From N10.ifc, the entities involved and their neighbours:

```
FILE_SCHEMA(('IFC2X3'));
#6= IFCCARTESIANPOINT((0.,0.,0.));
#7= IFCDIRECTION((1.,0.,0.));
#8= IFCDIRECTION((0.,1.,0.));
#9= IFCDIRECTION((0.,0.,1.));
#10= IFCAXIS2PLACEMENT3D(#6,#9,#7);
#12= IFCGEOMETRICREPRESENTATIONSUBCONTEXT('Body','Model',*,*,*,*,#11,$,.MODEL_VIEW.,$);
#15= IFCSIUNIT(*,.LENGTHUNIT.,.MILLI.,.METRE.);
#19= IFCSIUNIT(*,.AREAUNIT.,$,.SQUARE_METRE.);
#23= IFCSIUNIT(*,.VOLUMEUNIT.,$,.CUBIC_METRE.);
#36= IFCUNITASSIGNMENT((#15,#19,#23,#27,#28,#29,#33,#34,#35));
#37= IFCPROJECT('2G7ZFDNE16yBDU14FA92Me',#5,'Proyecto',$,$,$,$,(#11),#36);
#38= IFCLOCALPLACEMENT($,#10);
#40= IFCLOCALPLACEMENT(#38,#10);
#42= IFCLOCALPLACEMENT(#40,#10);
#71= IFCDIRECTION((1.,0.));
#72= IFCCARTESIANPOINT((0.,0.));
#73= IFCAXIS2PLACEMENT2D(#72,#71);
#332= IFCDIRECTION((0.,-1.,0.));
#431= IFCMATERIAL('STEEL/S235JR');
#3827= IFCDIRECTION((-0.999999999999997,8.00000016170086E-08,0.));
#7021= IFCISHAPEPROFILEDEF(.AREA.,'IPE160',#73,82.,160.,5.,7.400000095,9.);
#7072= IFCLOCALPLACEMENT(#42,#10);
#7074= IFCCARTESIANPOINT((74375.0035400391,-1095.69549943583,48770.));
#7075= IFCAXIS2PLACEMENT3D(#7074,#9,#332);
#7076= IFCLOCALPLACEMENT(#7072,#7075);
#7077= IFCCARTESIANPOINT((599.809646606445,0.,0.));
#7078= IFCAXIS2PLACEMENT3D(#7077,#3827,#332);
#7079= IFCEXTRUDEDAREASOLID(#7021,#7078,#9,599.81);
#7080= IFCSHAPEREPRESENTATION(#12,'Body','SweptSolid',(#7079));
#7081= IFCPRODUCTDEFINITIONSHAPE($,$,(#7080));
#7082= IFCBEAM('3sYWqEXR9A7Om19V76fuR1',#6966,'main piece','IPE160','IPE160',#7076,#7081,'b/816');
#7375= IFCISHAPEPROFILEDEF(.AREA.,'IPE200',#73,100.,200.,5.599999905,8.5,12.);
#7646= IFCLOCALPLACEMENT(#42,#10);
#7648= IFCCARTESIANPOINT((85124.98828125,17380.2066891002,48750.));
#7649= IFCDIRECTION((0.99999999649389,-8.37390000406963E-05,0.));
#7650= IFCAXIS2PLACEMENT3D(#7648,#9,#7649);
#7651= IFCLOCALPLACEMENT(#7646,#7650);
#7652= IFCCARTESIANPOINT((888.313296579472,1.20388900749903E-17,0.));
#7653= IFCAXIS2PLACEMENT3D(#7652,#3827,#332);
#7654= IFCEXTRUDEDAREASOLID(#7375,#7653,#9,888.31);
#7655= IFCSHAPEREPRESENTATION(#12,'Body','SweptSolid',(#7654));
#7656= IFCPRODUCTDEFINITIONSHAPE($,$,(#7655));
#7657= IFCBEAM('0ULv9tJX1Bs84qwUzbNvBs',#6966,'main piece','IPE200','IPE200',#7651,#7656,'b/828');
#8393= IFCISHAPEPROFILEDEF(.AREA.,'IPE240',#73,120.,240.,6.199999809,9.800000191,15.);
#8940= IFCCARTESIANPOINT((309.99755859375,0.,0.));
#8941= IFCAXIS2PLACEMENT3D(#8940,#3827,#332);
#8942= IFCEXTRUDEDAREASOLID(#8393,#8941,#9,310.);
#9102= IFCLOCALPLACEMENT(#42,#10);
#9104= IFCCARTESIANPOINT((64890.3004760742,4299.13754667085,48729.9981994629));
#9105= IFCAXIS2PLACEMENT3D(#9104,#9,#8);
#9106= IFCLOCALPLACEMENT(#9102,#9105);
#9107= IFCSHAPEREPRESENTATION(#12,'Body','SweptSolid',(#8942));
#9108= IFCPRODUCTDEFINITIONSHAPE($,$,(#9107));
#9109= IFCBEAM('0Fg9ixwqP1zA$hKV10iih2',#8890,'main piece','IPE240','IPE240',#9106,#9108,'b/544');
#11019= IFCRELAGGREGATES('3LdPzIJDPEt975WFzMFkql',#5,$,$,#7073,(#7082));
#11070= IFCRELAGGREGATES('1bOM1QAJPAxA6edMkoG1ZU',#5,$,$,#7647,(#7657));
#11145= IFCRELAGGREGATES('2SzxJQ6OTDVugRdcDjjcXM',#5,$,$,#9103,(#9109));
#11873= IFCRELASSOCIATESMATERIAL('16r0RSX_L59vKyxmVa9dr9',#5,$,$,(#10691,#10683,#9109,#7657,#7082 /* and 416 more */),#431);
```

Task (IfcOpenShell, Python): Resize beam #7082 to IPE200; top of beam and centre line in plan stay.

```python
import ifcopenshell
import ifcopenshell.util.element
import ifcopenshell.util.representation

model = ifcopenshell.open("N10.ifc")

member = model.by_guid("3sYWqEXR9A7Om19V76fuR1")
source = next(p for p in model.by_type("IfcIShapeProfileDef") if p.ProfileName == "IPE200")

body = ifcopenshell.util.representation.get_representation(member, "Model", "Body")
solid = body.Items[0]
old_profile = solid.SweptArea

# Copy the section's sizes but keep this member's own profile position.
profile = ifcopenshell.util.element.copy(model, source)
# Profiles are centred, so shift by half the change in depth to hold the top.
shift = (old_profile.OverallDepth - profile.OverallDepth) / 2
x, y = old_profile.Position.Location.Coordinates
up = (0.0, 1.0)  # upwards, in the solid's own plane
location = model.createIfcCartesianPoint((x + up[0] * shift, y + up[1] * shift))
profile.Position = model.createIfcAxis2Placement2D(location, old_profile.Position.RefDirection)
solid.SweptArea = profile
if not model.get_total_inverses(old_profile):
    ifcopenshell.util.element.remove_deep2(model, old_profile)
member.Description = member.Description.replace("IPE160", "IPE200")
member.ObjectType = member.ObjectType.replace("IPE160", "IPE200")

print(solid.SweptArea)

model.write("N10_v2.ifc")
```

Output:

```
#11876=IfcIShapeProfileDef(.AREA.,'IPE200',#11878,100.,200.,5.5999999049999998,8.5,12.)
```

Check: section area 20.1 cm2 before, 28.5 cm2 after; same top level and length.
